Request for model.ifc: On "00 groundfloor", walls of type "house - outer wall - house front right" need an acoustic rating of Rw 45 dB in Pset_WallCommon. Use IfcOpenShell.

First a look at what the model holds.

```python
import ifcopenshell
import ifcopenshell.util.element

model = ifcopenshell.open("model.ifc")
print(model.schema)
storey = next(s for s in model.by_type("IfcBuildingStorey") if s.Name == "00 groundfloor")
walls = [e for e in ifcopenshell.util.element.get_decomposition(storey) if e.is_a("IfcWall")]
seen = {}
for e in walls:
    element_type = ifcopenshell.util.element.get_type(e)
    key = (element_type.Name if element_type != e and element_type else None, ifcopenshell.util.element.get_pset(e, "Pset_WallCommon", "AcousticRating"))
    seen[key] = seen.get(key, 0) + 1
for (name, value), count in sorted(seen.items(), key=str):
    print(count, "x", name, "|", value)
```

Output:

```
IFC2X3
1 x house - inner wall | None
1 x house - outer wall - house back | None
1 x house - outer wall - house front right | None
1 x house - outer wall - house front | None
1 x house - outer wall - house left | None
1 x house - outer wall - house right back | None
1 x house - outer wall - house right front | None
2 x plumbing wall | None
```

```python
import ifcopenshell
import ifcopenshell.api.pset
import ifcopenshell.util.element

model = ifcopenshell.open("model.ifc")

storey = next(s for s in model.by_type("IfcBuildingStorey") if s.Name == "00 groundfloor")
walls = [e for e in ifcopenshell.util.element.get_decomposition(storey) if e.is_a("IfcWall")]

count = 0
for e in walls:
    element_type = ifcopenshell.util.element.get_type(e)
    if element_type in (None, e) or element_type.Name != "house - outer wall - house front right":
        continue
    # add_pset returns the element's existing set when there is one.
    pset = ifcopenshell.api.pset.add_pset(model, product=e, name="Pset_WallCommon")
    ifcopenshell.api.pset.edit_pset(model, pset=pset, properties={"AcousticRating": "Rw 45 dB"})
    count += 1

print(count, "walls updated")

model.write("model_updated.ifc")
```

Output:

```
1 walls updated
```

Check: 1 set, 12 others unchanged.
